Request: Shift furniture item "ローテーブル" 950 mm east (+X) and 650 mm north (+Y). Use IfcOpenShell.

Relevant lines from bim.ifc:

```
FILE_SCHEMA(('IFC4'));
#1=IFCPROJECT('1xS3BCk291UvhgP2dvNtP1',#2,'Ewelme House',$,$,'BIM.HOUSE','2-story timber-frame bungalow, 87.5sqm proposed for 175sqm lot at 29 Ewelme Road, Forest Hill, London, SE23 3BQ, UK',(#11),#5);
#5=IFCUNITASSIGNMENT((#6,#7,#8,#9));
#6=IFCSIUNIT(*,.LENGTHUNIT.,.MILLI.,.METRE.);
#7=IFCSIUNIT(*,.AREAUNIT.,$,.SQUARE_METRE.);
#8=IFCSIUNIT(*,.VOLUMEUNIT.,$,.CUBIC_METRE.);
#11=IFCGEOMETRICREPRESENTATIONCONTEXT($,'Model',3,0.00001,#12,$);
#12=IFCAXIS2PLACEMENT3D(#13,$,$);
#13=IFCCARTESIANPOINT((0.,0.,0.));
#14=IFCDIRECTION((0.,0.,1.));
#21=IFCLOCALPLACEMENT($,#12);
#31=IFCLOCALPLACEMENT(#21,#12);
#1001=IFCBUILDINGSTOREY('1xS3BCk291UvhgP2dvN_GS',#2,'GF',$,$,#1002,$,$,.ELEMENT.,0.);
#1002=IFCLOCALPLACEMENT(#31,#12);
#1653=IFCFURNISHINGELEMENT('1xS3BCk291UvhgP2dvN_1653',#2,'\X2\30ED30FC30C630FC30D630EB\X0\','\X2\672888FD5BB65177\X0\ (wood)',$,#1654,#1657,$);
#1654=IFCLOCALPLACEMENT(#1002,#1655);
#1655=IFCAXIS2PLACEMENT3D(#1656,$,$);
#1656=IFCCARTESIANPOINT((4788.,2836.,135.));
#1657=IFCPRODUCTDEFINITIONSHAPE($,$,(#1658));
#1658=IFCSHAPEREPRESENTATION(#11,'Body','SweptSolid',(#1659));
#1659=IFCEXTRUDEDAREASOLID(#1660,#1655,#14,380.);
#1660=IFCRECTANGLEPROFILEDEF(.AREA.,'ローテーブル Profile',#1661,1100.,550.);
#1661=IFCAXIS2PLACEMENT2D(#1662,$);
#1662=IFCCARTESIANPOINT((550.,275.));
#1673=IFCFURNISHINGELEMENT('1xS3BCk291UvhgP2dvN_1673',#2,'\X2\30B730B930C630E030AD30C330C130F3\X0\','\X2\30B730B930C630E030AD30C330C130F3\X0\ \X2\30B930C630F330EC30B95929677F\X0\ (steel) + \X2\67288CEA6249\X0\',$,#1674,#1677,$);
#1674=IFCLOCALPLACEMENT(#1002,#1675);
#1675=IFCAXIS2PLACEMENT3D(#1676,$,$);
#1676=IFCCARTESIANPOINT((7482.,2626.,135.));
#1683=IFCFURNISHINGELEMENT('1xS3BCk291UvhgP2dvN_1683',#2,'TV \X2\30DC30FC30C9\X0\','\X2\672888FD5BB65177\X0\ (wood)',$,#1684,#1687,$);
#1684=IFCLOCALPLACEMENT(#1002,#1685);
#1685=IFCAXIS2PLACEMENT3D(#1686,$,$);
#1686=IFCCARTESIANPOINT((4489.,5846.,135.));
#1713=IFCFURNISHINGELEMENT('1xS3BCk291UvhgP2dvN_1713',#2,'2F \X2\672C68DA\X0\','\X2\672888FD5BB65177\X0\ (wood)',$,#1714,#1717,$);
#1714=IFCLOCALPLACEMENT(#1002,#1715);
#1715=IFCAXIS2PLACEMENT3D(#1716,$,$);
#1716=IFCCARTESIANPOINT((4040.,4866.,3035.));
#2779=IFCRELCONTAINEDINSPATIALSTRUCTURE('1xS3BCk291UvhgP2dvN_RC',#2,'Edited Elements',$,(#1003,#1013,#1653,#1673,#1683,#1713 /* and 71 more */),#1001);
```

```python
import ifcopenshell
import ifcopenshell.api.geometry
import ifcopenshell.util.placement

model = ifcopenshell.open("bim.ifc")

item = model.by_guid("1xS3BCk291UvhgP2dvN_1653")
matrix = ifcopenshell.util.placement.get_local_placement(item.ObjectPlacement)
matrix[0, 3] += 950.0
matrix[1, 3] += 650.0
ifcopenshell.api.geometry.edit_object_placement(model, product=item, matrix=matrix, is_si=False)

print(ifcopenshell.util.placement.get_local_placement(item.ObjectPlacement).round(3) + 0.0)

model.write("bim_rev.ifc")
```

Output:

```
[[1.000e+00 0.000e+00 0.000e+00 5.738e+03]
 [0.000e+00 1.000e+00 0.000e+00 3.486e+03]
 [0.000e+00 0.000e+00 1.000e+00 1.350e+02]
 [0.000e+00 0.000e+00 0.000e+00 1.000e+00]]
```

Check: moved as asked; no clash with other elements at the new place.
